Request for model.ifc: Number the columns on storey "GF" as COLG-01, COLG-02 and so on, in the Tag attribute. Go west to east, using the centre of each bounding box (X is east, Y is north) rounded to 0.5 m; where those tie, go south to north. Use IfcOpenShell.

First a look at what the model holds.

```python
import ifcopenshell
import ifcopenshell.util.element
import ifcopenshell.util.placement

model = ifcopenshell.open("model.ifc")
print(model.schema)
storey = next(s for s in model.by_type("IfcBuildingStorey") if s.Name == "GF")
columns = [e for e in ifcopenshell.util.element.get_decomposition(storey) if e.is_a("IfcColumn")]
for e in sorted(columns, key=lambda e: e.id()):
    origin = ifcopenshell.util.placement.get_local_placement(e.ObjectPlacement)[:3, 3]
    print(e.id(), e.Tag, e.Name, origin.round(2) + 0.0, sep=" | ")
```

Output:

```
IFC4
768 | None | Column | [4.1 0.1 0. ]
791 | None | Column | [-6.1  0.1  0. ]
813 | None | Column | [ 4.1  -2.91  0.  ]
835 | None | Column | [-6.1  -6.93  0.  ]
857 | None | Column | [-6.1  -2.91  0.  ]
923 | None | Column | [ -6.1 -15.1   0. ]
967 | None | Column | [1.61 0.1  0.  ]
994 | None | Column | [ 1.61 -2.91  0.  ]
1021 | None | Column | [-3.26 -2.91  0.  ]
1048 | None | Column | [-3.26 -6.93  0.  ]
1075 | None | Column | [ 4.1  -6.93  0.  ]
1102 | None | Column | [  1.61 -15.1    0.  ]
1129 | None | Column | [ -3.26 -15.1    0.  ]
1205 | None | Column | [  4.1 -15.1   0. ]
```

```python
import ifcopenshell
import ifcopenshell.geom
import ifcopenshell.util.element
import ifcopenshell.util.shape

model = ifcopenshell.open("model.ifc")
settings = ifcopenshell.geom.settings()
settings.set("use-world-coords", True)


def centre(element):
    shape = ifcopenshell.geom.create_shape(settings, element)
    return ifcopenshell.util.shape.get_bbox_centroid(shape.geometry)


storey = next(s for s in model.by_type("IfcBuildingStorey") if s.Name == "GF")
columns = [e for e in ifcopenshell.util.element.get_decomposition(storey) if e.is_a("IfcColumn")]

# Insertion points can sit at a corner or the storey origin, so sort by the geometry (in metres).
centres = {e: centre(e) for e in columns}
columns.sort(key=lambda e: (round(centres[e][0] / 0.5), centres[e][1]))

for i, e in enumerate(columns, start=1):
    number = f"COLG-{i:02d}"
    e.Tag = number
    print(e.id(), number)

model.write("model_v2.ifc")
```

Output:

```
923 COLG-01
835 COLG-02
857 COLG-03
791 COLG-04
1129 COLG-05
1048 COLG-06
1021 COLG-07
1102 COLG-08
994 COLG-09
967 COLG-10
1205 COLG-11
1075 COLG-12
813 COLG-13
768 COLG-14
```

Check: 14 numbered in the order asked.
